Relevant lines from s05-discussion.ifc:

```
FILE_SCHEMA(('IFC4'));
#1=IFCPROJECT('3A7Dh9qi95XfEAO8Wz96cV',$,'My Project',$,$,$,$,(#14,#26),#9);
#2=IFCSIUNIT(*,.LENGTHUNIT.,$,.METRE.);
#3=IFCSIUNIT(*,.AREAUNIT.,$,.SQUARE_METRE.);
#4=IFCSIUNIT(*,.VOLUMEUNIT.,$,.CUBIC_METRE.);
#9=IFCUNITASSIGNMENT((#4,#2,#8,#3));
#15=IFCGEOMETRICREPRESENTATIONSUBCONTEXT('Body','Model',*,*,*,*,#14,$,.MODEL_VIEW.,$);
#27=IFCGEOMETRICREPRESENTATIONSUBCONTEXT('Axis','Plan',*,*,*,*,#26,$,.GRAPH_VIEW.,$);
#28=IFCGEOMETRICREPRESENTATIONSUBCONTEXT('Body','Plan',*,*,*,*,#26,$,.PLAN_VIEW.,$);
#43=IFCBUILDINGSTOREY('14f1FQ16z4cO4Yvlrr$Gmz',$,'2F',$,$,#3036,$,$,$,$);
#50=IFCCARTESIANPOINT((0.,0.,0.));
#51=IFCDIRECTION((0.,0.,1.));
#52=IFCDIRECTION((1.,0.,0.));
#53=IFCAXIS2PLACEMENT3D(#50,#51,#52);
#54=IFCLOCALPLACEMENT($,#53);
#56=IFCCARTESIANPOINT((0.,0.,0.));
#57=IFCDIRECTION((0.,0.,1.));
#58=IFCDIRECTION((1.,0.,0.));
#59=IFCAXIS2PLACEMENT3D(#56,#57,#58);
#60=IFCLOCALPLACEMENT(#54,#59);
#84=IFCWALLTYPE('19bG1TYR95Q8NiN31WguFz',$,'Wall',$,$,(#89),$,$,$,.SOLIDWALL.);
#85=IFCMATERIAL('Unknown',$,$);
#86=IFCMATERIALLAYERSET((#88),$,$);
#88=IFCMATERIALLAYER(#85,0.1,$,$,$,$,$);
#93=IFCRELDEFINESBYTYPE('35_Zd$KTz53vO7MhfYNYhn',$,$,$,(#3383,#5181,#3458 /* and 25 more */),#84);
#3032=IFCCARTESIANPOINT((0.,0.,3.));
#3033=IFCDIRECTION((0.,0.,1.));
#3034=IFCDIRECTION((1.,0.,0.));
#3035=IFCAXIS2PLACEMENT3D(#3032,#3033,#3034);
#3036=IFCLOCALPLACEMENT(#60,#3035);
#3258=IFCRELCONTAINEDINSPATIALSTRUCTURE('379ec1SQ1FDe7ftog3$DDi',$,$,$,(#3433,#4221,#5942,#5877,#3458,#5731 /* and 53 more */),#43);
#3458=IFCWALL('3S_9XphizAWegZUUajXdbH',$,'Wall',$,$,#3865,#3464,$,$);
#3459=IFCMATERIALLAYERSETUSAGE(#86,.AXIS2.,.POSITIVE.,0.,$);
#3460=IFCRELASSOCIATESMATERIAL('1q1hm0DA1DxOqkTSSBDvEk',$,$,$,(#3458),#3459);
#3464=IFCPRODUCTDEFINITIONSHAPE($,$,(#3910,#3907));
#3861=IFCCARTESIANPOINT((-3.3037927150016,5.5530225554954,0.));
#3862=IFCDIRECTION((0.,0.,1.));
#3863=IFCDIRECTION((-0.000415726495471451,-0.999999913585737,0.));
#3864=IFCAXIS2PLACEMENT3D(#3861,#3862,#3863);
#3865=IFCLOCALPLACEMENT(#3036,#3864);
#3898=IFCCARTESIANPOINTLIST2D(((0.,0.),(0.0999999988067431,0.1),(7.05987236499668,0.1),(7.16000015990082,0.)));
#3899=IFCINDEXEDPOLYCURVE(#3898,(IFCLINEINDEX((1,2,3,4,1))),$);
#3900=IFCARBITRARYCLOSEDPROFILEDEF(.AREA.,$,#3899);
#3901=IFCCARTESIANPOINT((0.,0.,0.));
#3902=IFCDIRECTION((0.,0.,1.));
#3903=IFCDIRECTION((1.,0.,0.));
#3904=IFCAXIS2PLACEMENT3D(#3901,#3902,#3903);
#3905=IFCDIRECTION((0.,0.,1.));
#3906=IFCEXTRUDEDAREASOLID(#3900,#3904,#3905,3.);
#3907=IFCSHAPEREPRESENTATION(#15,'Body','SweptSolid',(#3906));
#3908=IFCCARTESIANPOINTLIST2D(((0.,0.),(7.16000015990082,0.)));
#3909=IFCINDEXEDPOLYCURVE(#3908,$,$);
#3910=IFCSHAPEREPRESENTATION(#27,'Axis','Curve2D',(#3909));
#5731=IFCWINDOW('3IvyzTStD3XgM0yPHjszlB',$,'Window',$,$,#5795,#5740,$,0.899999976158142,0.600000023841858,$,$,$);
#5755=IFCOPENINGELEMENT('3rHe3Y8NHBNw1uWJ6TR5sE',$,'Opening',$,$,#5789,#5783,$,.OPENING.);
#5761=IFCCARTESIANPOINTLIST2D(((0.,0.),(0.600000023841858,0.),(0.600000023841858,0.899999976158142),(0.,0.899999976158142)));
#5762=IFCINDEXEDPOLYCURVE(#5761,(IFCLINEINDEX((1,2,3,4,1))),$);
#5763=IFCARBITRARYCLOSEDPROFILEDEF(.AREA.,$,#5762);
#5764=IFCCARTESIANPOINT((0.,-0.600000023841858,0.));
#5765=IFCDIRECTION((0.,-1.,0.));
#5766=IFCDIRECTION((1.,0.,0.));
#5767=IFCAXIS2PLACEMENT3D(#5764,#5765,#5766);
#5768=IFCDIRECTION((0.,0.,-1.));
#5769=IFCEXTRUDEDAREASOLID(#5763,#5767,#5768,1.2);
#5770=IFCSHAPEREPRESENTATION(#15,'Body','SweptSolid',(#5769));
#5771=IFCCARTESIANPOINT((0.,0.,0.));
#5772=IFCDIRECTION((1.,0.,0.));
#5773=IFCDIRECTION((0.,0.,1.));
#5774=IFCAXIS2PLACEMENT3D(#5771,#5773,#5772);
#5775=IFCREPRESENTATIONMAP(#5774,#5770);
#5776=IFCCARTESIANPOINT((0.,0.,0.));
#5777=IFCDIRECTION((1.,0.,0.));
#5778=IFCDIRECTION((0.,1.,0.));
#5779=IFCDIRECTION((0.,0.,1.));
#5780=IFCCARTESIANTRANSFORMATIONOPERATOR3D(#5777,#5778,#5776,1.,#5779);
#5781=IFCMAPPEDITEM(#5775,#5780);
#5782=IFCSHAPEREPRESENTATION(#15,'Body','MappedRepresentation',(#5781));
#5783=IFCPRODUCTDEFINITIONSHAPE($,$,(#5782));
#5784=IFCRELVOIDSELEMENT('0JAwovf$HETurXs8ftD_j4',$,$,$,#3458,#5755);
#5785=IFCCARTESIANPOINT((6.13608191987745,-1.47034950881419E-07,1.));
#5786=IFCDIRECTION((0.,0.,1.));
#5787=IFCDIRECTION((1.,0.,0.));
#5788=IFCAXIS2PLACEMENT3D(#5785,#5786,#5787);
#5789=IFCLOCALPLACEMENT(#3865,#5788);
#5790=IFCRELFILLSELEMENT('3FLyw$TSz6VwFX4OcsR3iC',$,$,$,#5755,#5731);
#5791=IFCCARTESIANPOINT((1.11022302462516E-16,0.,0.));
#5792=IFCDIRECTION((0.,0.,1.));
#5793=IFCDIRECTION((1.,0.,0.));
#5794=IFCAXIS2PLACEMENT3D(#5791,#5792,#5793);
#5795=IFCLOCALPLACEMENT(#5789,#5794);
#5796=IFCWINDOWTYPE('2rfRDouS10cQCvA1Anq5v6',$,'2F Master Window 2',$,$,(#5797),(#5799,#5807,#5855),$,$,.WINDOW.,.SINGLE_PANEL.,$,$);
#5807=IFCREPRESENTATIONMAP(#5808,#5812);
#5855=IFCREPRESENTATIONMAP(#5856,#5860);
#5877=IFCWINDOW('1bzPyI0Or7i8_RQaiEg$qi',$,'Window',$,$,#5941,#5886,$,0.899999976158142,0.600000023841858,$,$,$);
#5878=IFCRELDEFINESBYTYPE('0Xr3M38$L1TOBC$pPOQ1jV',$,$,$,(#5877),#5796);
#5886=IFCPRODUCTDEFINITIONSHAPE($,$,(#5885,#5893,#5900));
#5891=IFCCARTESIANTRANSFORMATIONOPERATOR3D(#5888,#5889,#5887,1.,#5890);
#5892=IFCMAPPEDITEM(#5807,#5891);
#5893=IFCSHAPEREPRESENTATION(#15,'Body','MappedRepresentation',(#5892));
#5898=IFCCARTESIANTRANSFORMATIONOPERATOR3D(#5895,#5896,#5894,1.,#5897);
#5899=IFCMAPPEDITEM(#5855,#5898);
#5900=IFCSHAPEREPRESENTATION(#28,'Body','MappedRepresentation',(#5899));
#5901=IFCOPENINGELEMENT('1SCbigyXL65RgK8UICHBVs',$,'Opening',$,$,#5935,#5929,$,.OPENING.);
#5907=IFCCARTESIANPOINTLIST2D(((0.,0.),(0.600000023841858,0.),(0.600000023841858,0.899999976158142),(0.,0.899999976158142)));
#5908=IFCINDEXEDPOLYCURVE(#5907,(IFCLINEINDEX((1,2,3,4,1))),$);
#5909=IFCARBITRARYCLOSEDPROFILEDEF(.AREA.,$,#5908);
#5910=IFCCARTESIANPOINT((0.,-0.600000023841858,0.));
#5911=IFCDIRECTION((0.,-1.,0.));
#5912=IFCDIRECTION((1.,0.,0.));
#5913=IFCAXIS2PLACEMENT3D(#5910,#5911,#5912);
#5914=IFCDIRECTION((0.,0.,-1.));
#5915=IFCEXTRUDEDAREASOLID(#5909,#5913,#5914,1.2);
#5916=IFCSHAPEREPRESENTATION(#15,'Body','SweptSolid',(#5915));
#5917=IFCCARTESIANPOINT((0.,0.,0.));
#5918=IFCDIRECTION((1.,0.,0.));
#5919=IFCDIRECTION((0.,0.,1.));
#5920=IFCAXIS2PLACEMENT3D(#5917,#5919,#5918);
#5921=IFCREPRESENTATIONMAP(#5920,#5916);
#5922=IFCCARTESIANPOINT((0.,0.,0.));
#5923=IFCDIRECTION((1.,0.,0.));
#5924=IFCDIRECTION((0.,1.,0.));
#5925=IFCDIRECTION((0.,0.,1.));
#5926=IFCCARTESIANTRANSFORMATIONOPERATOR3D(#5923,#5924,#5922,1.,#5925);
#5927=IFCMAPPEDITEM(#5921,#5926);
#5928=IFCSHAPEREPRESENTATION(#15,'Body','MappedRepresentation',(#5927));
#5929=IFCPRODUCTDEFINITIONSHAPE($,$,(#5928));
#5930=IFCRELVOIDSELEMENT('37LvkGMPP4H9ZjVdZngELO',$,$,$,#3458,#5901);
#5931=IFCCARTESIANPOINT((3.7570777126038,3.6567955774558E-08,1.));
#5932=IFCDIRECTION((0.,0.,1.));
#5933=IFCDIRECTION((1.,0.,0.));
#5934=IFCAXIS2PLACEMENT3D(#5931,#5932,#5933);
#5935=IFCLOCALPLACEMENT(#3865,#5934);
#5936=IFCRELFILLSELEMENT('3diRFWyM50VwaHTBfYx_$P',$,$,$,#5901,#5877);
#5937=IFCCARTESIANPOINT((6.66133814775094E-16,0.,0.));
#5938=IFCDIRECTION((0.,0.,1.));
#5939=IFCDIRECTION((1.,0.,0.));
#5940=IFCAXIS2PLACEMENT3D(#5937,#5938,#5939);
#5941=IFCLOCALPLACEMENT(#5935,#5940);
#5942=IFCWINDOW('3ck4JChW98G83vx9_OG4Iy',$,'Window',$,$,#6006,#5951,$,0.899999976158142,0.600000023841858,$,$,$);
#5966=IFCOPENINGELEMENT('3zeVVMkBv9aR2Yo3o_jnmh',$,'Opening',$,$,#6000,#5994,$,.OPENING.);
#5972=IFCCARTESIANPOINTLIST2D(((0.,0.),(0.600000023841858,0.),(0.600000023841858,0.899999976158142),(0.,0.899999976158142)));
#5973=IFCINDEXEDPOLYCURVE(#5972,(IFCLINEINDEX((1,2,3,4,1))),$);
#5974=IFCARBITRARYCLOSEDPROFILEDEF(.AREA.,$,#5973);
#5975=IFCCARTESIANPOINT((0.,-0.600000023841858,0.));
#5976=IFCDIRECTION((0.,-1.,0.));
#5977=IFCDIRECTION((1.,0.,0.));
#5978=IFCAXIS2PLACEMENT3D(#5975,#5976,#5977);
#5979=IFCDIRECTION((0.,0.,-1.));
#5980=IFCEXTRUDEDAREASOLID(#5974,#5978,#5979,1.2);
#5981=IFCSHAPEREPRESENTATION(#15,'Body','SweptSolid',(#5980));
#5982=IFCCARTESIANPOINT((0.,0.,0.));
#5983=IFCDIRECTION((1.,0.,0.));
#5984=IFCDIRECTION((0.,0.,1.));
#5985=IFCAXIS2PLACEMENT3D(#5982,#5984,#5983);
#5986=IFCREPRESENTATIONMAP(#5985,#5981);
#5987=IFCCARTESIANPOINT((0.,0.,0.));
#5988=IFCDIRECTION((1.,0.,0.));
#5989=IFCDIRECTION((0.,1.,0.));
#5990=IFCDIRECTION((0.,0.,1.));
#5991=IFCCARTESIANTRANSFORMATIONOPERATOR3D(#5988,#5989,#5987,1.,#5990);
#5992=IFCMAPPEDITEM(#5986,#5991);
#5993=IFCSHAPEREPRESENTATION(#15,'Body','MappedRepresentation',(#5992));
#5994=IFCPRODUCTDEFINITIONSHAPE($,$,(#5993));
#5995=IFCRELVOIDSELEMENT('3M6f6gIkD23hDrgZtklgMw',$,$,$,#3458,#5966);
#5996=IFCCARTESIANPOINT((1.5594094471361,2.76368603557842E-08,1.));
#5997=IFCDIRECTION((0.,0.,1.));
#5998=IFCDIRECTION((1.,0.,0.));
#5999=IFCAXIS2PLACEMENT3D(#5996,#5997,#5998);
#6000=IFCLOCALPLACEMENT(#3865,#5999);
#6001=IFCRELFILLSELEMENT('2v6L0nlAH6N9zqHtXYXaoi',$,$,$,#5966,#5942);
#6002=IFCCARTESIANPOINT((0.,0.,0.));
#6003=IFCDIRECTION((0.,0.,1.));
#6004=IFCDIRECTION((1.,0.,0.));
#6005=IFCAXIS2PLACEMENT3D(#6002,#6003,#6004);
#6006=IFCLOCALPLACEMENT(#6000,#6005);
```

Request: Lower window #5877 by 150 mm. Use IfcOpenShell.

```python
import numpy as np
import ifcopenshell
import ifcopenshell.api.geometry
import ifcopenshell.util.placement
import ifcopenshell.util.unit

model = ifcopenshell.open("s05-discussion.ifc")
unit_scale = ifcopenshell.util.unit.calculate_unit_scale(model)

window = model.by_id(5877)
opening = window.FillsVoids[0].RelatingOpeningElement
dz = -0.15

shift = np.array([0.0, 0.0, dz])
# The window is placed relative to its opening, so it follows when the opening moves.
matrix = ifcopenshell.util.placement.get_local_placement(opening.ObjectPlacement)
matrix[:3, 3] += shift
ifcopenshell.api.geometry.edit_object_placement(
    model, product=opening, matrix=matrix, is_si=False, should_transform_children=True
)

print(f"moved by {dz * unit_scale:+.3f} m")

model.write("s05-discussion_updated.ifc")
```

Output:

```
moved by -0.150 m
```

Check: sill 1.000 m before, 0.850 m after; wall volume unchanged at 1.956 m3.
